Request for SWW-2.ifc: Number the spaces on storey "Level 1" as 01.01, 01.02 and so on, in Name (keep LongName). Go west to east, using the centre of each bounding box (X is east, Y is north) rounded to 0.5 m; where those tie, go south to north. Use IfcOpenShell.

First a look at what the model holds.

```python
import ifcopenshell
import ifcopenshell.util.element
import ifcopenshell.util.placement

model = ifcopenshell.open("SWW-2.ifc")
print(model.schema)
storey = next(s for s in model.by_type("IfcBuildingStorey") if s.Name == "Level 1")
spaces = [e for e in ifcopenshell.util.element.get_decomposition(storey) if e.is_a("IfcSpace")]
for e in sorted(spaces, key=lambda e: e.id()):
    origin = ifcopenshell.util.placement.get_local_placement(e.ObjectPlacement)[:3, 3]
    print(e.id(), e.Name, e.LongName, origin.round(2) + 0.0, sep=" | ")
```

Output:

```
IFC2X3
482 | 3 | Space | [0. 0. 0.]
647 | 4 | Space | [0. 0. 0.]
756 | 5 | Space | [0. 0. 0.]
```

```python
import ifcopenshell
import ifcopenshell.geom
import ifcopenshell.util.element
import ifcopenshell.util.shape

model = ifcopenshell.open("SWW-2.ifc")
settings = ifcopenshell.geom.settings()
settings.set("use-world-coords", True)


def centre(element):
    shape = ifcopenshell.geom.create_shape(settings, element)
    return ifcopenshell.util.shape.get_bbox_centroid(shape.geometry)


storey = next(s for s in model.by_type("IfcBuildingStorey") if s.Name == "Level 1")
spaces = [e for e in ifcopenshell.util.element.get_decomposition(storey) if e.is_a("IfcSpace")]

# Insertion points can sit at a corner or the storey origin, so sort by the geometry (in metres).
centres = {e: centre(e) for e in spaces}
spaces.sort(key=lambda e: (round(centres[e][0] / 0.5), centres[e][1]))

for i, e in enumerate(spaces, start=1):
    number = f"01.{i:02d}"
    e.Name = number
    print(e.id(), number)

model.write("SWW-2_updated.ifc")
```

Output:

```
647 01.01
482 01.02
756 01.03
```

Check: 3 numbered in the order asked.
